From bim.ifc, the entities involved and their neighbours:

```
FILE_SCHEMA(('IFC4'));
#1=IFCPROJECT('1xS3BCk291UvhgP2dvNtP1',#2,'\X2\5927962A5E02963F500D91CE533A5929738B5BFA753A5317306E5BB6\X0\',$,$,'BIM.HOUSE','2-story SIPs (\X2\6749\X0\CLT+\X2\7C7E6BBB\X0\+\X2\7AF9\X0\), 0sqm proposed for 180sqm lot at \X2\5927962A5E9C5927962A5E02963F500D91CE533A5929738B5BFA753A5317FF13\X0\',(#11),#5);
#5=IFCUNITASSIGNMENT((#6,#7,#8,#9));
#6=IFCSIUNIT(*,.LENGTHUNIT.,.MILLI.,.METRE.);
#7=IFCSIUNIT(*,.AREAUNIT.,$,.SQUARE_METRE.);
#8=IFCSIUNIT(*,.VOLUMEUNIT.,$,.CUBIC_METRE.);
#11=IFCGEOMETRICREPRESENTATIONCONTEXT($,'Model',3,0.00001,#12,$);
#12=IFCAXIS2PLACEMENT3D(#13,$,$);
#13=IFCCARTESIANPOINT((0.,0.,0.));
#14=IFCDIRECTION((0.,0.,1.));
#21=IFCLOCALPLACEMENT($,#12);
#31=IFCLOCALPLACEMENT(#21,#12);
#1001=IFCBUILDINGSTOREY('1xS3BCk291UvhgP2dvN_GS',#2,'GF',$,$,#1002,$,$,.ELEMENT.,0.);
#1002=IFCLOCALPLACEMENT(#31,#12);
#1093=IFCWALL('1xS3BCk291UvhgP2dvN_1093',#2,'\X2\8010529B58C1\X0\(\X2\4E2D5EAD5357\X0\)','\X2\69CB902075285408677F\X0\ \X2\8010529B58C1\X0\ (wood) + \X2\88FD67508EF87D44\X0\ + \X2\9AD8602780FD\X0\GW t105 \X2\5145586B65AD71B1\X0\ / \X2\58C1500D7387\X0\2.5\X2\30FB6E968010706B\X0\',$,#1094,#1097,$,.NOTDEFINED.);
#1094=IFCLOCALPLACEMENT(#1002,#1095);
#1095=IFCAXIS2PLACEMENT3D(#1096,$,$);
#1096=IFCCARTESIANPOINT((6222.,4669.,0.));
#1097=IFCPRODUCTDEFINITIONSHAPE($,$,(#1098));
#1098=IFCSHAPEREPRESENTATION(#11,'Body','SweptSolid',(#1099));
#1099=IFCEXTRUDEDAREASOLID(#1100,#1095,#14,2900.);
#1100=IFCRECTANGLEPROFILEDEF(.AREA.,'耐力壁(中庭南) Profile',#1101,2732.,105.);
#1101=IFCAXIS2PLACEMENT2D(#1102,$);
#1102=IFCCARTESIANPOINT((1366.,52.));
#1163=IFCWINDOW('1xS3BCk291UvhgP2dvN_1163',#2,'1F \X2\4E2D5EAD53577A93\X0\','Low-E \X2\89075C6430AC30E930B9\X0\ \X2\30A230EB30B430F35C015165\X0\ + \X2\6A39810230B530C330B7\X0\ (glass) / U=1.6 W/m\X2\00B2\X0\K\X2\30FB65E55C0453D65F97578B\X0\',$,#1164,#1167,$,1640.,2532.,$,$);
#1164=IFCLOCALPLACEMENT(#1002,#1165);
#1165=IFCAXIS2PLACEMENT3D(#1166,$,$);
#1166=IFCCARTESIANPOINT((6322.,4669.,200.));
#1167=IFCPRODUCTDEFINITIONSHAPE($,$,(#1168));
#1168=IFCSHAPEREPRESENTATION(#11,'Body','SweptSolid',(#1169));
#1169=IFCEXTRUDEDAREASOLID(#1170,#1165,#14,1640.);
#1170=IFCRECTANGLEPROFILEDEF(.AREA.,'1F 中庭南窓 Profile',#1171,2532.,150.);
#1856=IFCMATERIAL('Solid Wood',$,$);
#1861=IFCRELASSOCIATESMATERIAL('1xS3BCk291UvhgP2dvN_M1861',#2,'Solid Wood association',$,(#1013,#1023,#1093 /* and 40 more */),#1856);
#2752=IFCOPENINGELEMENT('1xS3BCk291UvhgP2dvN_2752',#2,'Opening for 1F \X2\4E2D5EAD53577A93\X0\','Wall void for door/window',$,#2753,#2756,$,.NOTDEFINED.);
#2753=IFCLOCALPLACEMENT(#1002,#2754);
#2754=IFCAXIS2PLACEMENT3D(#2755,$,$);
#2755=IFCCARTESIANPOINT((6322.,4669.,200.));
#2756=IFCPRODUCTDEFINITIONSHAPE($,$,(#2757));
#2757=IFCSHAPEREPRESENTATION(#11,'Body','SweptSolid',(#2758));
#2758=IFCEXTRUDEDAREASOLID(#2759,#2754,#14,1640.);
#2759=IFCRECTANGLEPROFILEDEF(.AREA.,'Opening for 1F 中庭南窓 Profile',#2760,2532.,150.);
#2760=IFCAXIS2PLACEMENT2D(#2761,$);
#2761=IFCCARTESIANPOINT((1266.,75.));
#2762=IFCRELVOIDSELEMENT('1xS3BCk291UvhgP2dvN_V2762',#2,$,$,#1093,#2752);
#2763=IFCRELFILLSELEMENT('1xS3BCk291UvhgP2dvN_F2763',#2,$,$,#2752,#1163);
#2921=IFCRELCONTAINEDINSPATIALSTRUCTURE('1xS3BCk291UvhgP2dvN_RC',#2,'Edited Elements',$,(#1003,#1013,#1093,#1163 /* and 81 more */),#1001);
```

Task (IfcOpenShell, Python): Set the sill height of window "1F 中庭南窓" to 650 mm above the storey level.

```python
import numpy as np
import ifcopenshell
import ifcopenshell.api.geometry
import ifcopenshell.geom
import ifcopenshell.util.element
import ifcopenshell.util.placement
import ifcopenshell.util.shape
import ifcopenshell.util.unit

model = ifcopenshell.open("bim.ifc")
unit_scale = ifcopenshell.util.unit.calculate_unit_scale(model)

window = model.by_guid("1xS3BCk291UvhgP2dvN_1163")
opening = window.FillsVoids[0].RelatingOpeningElement
storey = ifcopenshell.util.element.get_container(window, ifc_class="IfcBuildingStorey")
level = ifcopenshell.util.placement.get_local_placement(storey.ObjectPlacement)[2, 3]

# The opening's origin need not be at the sill, so measure its lowest point.
shape = ifcopenshell.geom.create_shape(ifcopenshell.geom.settings(), opening)
bottom = ifcopenshell.util.shape.get_shape_bottom_elevation(shape, shape.geometry) / unit_scale
dz = level + 650.0 - bottom

shift = np.array([0.0, 0.0, dz])
# The window is not placed relative to its opening, so move both.
for product in (opening, window):
    matrix = ifcopenshell.util.placement.get_local_placement(product.ObjectPlacement)
    matrix[:3, 3] += shift
    ifcopenshell.api.geometry.edit_object_placement(model, product=product, matrix=matrix, is_si=False)

print(f"moved by {dz * unit_scale:+.3f} m")

model.write("bim-out.ifc")
```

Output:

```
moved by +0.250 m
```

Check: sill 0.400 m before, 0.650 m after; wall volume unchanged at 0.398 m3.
